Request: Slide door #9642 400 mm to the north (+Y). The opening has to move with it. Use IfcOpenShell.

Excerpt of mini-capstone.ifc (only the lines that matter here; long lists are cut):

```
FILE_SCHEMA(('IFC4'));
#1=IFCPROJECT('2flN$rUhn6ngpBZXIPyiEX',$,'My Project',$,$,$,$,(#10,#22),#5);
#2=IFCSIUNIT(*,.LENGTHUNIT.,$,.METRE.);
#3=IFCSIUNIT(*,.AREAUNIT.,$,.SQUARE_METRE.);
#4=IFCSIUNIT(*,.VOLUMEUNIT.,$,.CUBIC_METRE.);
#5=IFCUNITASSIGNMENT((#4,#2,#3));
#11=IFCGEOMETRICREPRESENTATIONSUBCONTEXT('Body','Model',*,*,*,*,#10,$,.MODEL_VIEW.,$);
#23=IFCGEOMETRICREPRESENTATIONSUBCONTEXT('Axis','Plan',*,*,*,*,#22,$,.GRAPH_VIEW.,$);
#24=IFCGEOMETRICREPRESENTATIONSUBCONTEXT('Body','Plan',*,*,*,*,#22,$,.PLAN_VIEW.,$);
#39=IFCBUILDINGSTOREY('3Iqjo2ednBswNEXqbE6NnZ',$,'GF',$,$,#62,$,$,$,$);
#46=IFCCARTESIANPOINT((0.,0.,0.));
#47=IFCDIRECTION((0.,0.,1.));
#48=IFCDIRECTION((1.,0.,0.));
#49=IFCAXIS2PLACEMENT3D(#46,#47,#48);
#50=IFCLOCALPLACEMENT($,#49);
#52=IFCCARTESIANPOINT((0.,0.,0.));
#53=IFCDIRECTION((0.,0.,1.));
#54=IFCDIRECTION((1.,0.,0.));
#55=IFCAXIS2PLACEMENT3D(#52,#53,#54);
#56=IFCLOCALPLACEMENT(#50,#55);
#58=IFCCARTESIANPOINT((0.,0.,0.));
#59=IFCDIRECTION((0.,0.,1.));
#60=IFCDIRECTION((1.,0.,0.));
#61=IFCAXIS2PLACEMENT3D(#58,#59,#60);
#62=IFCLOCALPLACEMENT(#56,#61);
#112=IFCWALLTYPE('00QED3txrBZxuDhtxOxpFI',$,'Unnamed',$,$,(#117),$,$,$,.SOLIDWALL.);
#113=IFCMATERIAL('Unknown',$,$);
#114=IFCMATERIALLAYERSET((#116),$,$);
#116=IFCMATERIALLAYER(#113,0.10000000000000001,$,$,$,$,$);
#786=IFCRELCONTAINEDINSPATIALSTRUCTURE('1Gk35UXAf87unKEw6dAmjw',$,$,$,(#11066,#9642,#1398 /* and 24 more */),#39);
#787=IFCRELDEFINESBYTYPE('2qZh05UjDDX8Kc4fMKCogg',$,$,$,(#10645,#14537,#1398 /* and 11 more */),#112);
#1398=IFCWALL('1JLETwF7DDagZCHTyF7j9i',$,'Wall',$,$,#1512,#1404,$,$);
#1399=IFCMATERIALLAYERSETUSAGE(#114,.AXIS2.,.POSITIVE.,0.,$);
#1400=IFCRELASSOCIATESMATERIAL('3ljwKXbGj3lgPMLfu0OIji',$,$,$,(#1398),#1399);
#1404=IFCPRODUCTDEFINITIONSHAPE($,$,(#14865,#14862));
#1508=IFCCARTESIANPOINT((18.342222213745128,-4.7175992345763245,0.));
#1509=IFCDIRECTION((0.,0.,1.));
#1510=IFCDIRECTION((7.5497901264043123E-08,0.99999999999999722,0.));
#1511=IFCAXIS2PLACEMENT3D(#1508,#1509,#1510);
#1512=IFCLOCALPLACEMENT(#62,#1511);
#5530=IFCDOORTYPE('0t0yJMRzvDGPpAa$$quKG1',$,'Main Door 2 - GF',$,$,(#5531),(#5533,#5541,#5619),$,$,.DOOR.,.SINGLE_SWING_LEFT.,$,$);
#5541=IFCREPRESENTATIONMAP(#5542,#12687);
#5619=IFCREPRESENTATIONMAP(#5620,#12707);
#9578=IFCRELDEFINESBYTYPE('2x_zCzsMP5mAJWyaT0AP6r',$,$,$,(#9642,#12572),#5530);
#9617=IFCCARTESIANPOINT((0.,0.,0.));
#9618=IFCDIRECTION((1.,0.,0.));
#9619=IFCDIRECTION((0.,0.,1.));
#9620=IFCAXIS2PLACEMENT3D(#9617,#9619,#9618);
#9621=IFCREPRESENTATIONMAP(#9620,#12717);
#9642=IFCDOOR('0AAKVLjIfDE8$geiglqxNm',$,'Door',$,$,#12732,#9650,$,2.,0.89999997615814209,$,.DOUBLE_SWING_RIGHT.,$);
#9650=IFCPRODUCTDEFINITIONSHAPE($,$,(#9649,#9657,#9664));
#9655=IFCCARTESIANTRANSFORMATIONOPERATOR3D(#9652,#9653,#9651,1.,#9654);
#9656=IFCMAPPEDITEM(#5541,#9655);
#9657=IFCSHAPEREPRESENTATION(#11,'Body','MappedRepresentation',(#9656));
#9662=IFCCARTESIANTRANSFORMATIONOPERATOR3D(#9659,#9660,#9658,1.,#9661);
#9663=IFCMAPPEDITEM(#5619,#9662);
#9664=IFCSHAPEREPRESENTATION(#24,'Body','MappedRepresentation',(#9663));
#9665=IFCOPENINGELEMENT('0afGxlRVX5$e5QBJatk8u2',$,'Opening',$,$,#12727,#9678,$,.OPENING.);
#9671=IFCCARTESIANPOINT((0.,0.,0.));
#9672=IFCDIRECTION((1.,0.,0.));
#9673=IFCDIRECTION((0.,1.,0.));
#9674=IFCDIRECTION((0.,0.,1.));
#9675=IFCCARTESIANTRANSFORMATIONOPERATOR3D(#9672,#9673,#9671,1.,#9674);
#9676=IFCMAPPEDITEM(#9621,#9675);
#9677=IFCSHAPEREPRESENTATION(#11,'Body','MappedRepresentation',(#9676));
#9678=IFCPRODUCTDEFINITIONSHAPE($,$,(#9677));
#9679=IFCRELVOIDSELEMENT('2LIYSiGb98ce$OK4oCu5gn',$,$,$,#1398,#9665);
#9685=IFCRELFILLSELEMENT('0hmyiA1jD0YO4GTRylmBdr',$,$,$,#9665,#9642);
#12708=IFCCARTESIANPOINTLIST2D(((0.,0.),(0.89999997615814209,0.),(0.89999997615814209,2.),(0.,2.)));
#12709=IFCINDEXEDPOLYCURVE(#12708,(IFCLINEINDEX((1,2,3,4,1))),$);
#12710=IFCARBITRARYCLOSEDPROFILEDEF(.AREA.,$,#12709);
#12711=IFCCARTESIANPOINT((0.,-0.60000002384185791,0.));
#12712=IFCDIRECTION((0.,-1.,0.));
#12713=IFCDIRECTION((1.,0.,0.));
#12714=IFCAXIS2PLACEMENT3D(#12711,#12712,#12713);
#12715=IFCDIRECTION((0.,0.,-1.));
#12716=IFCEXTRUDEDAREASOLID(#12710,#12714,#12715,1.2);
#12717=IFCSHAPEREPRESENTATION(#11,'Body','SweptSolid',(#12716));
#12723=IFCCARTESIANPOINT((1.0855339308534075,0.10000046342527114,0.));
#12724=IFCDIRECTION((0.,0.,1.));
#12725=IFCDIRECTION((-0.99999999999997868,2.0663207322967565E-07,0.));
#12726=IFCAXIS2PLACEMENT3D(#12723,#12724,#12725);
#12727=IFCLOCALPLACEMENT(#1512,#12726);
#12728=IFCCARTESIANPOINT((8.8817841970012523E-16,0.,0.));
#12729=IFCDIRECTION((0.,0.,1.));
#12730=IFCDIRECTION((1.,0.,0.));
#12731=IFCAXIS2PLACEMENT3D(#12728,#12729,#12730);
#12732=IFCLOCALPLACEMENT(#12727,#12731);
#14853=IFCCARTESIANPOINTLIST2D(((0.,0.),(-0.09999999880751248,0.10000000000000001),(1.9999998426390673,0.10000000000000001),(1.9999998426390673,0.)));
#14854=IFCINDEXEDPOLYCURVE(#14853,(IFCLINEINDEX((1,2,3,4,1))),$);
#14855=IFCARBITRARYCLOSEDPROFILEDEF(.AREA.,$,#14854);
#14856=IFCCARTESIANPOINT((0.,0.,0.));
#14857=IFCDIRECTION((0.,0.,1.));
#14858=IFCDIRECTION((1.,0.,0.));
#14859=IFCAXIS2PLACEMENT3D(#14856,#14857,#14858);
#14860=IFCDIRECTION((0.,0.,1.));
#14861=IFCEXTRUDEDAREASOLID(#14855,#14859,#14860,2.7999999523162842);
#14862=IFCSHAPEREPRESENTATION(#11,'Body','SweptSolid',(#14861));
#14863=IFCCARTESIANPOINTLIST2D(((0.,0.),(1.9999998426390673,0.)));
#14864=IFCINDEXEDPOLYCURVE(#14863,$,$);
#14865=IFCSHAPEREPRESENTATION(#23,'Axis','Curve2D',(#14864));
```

```python
import ifcopenshell
import ifcopenshell.api.geometry
import ifcopenshell.util.placement

model = ifcopenshell.open("mini-capstone.ifc")

door = model.by_guid("0AAKVLjIfDE8$geiglqxNm")
opening = door.FillsVoids[0].RelatingOpeningElement
wall = opening.VoidsElements[0].RelatingBuildingElement

wall_matrix = ifcopenshell.util.placement.get_local_placement(wall.ObjectPlacement)
shift = wall_matrix[:3, 0] * 0.4
before = ifcopenshell.util.placement.get_local_placement(door.ObjectPlacement)[:3, 3].copy()

# The door is placed relative to its opening, so it follows when the opening moves.
matrix = ifcopenshell.util.placement.get_local_placement(opening.ObjectPlacement)
matrix[:3, 3] += shift
ifcopenshell.api.geometry.edit_object_placement(
    model, product=opening, matrix=matrix, is_si=False, should_transform_children=True
)

after = ifcopenshell.util.placement.get_local_placement(door.ObjectPlacement)[:3, 3]
print("door moved by", (after - before).round(3) + 0.0)

model.write("mini-capstone_updated.ifc")
```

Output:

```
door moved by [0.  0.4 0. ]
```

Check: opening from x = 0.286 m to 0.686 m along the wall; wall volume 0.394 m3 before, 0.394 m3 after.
